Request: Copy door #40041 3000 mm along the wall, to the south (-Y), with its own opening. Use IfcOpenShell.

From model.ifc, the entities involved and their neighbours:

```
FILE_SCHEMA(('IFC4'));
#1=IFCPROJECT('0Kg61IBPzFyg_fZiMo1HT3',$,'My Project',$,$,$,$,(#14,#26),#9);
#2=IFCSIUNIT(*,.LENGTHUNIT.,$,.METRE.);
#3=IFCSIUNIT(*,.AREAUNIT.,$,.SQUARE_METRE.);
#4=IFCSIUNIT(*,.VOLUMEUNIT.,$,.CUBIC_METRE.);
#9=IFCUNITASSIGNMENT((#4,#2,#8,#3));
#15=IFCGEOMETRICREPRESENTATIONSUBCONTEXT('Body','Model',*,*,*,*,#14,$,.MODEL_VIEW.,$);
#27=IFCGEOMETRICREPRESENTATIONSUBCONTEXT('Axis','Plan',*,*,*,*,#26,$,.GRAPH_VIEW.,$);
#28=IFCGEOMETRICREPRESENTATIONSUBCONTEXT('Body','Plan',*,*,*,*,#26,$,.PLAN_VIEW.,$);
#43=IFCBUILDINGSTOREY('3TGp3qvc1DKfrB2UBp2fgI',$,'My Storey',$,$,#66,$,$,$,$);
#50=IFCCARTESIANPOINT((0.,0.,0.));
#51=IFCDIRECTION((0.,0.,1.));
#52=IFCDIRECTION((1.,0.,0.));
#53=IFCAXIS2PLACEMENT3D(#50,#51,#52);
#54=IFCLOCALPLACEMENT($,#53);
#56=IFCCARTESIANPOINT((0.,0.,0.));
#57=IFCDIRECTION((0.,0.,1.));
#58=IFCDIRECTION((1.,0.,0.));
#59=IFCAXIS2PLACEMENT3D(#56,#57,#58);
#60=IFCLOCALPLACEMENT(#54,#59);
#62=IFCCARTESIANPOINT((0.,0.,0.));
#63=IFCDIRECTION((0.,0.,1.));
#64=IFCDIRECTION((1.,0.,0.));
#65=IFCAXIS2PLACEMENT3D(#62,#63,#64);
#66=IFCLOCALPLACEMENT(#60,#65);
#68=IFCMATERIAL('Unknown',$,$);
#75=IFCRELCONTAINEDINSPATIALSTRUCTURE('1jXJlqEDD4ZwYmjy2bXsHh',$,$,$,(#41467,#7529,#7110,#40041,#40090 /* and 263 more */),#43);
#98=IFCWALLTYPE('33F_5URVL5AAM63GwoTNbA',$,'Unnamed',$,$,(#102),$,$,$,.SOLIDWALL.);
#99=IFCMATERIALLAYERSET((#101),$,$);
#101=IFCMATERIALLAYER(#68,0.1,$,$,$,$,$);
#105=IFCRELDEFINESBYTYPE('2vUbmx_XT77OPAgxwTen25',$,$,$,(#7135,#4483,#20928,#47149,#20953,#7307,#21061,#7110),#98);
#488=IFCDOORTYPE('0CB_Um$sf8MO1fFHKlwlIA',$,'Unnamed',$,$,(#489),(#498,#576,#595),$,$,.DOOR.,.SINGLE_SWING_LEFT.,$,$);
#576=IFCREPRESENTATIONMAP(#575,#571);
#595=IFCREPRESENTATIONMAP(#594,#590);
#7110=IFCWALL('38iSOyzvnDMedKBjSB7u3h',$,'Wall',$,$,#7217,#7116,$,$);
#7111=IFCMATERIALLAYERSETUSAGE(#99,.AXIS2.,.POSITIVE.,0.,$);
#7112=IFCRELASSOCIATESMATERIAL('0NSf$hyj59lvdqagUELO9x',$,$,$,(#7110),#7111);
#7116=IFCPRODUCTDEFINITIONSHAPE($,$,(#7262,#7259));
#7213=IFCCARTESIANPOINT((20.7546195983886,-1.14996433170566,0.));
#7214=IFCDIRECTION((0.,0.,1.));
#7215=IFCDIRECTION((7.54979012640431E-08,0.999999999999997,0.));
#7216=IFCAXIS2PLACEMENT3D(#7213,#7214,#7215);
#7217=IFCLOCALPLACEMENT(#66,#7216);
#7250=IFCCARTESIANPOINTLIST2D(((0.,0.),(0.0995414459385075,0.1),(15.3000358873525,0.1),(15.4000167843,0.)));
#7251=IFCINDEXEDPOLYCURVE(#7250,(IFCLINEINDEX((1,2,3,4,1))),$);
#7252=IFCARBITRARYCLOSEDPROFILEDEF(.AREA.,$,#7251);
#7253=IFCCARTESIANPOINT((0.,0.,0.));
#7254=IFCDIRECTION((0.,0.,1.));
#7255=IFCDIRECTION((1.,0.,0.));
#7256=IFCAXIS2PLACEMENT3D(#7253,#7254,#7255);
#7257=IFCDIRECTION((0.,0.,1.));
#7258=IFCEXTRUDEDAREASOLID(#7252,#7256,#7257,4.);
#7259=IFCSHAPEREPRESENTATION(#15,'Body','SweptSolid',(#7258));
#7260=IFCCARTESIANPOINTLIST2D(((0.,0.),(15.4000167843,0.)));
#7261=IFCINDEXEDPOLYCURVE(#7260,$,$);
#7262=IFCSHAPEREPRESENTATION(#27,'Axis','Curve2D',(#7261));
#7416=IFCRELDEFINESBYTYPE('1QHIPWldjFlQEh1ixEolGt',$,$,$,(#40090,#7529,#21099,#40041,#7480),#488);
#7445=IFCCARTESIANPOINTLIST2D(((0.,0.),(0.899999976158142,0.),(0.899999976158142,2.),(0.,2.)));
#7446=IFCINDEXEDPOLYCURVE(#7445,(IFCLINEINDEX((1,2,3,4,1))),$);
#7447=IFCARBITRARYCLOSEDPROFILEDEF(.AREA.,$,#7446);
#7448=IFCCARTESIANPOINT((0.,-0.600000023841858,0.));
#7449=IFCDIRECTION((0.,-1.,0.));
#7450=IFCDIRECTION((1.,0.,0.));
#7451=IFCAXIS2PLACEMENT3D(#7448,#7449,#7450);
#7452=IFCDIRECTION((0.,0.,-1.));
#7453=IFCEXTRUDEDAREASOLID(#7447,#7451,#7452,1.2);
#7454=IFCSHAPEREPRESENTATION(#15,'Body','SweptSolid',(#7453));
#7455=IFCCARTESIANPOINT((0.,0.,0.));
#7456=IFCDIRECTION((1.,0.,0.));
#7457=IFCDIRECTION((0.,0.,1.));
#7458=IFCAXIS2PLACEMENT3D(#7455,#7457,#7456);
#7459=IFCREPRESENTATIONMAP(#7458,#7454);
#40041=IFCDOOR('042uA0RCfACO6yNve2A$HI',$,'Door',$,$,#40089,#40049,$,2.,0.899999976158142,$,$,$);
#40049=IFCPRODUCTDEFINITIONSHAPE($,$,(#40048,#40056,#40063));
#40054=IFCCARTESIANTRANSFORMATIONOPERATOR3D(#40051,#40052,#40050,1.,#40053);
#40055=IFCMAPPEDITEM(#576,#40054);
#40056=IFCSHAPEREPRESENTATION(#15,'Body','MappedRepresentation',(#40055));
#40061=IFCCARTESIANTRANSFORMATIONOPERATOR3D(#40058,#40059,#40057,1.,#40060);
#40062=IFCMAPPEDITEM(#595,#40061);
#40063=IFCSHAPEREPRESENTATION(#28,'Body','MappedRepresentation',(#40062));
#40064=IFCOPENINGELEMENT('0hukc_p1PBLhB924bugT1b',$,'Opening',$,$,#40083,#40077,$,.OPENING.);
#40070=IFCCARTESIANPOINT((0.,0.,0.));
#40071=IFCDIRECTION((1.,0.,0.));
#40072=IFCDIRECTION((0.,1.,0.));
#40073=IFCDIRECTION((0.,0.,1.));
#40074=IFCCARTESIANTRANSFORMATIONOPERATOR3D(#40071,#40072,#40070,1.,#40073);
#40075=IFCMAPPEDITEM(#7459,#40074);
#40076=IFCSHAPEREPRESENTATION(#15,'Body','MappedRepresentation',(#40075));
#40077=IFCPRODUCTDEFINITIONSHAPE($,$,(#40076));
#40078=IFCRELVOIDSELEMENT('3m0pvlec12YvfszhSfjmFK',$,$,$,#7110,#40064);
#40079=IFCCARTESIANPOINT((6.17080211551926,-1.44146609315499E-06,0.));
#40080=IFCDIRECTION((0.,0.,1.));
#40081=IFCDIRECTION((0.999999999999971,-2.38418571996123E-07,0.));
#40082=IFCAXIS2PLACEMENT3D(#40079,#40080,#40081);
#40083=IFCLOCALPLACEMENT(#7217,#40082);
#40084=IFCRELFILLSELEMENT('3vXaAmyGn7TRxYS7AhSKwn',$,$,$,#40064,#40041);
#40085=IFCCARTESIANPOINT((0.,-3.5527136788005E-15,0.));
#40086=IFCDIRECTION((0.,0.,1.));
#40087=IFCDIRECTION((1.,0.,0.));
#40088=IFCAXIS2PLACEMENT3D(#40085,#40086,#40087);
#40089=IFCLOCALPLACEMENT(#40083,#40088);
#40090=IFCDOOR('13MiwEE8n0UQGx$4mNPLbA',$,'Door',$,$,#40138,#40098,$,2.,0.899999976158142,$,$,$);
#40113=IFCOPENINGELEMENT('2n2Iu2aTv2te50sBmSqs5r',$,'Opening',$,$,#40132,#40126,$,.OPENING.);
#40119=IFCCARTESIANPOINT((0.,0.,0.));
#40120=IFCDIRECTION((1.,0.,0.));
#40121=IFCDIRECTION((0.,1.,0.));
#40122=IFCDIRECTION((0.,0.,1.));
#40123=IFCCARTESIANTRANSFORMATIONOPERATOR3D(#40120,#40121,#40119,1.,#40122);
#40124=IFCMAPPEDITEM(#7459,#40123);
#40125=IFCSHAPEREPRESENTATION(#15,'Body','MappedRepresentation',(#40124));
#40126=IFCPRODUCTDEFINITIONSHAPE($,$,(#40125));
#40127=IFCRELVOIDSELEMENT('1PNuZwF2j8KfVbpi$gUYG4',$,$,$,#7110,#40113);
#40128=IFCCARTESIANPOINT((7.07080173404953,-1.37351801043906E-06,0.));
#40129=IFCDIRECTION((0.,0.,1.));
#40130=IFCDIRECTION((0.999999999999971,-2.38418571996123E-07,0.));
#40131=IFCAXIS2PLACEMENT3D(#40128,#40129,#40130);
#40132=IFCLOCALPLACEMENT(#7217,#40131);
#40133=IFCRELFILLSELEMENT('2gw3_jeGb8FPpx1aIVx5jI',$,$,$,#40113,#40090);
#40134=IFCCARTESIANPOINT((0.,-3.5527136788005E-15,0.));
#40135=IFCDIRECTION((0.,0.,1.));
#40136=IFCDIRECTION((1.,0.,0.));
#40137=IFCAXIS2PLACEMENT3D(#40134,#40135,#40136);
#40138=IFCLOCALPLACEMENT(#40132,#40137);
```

```python
import ifcopenshell
import ifcopenshell.api.feature
import ifcopenshell.api.geometry
import ifcopenshell.api.root
import ifcopenshell.geom
import ifcopenshell.util.element
import ifcopenshell.util.placement
import ifcopenshell.util.shape

model = ifcopenshell.open("model.ifc")
settings = ifcopenshell.geom.settings()


def volume(element):
    """Net volume in cubic metres, openings subtracted."""
    shape = ifcopenshell.geom.create_shape(settings, element)
    return ifcopenshell.util.shape.get_volume(shape.geometry)


door = model.by_guid("042uA0RCfACO6yNve2A$HI")
opening = door.FillsVoids[0].RelatingOpeningElement
wall = opening.VoidsElements[0].RelatingBuildingElement
before = volume(wall)
shift = ifcopenshell.util.placement.get_local_placement(wall.ObjectPlacement)[:3, 0] * -3.0

# copy_class copies the void relationship, type, container and properties, but no geometry.
new_opening = ifcopenshell.api.root.copy_class(model, product=opening)
new_opening.Representation = ifcopenshell.util.element.copy_deep(
    model, opening.Representation, exclude=["IfcGeometricRepresentationContext", "IfcRepresentationMap"]
)
new_door = ifcopenshell.api.root.copy_class(model, product=door)
new_door.Representation = ifcopenshell.util.element.copy_deep(
    model, door.Representation, exclude=["IfcGeometricRepresentationContext", "IfcRepresentationMap"]
)
ifcopenshell.api.feature.add_filling(model, opening=new_opening, element=new_door)

for old, new in ((opening, new_opening), (door, new_door)):
    matrix = ifcopenshell.util.placement.get_local_placement(old.ObjectPlacement)
    matrix[:3, 3] += shift
    ifcopenshell.api.geometry.edit_object_placement(model, product=new, matrix=matrix, is_si=False)

after = volume(wall)

print(f"wall volume {before:.3f} -> {after:.3f} m3")

model.write("model_v2.ifc")
```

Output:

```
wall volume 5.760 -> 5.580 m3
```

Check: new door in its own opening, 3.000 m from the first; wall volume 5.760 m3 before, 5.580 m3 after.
